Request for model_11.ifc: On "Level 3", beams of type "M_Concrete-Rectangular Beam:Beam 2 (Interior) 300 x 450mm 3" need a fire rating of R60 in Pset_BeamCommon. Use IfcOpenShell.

First a look at what the model holds.

```python
import ifcopenshell
import ifcopenshell.util.element

model = ifcopenshell.open("model_11.ifc")
print(model.schema)
storey = next(s for s in model.by_type("IfcBuildingStorey") if s.Name == "Level 3")
beams = [e for e in ifcopenshell.util.element.get_decomposition(storey) if e.is_a("IfcBeam")]
seen = {}
for e in beams:
    element_type = ifcopenshell.util.element.get_type(e)
    key = (element_type.Name if element_type != e and element_type else None, ifcopenshell.util.element.get_pset(e, "Pset_BeamCommon", "FireRating"))
    seen[key] = seen.get(key, 0) + 1
for (name, value), count in sorted(seen.items(), key=str):
    print(count, "x", name, "|", value)
```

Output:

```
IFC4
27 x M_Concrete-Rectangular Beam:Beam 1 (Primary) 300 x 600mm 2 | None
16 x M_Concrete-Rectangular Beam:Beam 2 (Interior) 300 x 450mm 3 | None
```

```python
import ifcopenshell
import ifcopenshell.api.pset
import ifcopenshell.util.element

model = ifcopenshell.open("model_11.ifc")

storey = next(s for s in model.by_type("IfcBuildingStorey") if s.Name == "Level 3")
beams = [e for e in ifcopenshell.util.element.get_decomposition(storey) if e.is_a("IfcBeam")]

count = 0
for e in beams:
    element_type = ifcopenshell.util.element.get_type(e)
    if element_type in (None, e) or element_type.Name != "M_Concrete-Rectangular Beam:Beam 2 (Interior) 300 x 450mm 3":
        continue
    # add_pset returns the element's existing set when there is one.
    pset = ifcopenshell.api.pset.add_pset(model, product=e, name="Pset_BeamCommon")
    ifcopenshell.api.pset.edit_pset(model, pset=pset, properties={"FireRating": "R60"})
    count += 1

print(count, "beams updated")

model.write("model_11_updated.ifc")
```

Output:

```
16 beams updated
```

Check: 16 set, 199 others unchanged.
